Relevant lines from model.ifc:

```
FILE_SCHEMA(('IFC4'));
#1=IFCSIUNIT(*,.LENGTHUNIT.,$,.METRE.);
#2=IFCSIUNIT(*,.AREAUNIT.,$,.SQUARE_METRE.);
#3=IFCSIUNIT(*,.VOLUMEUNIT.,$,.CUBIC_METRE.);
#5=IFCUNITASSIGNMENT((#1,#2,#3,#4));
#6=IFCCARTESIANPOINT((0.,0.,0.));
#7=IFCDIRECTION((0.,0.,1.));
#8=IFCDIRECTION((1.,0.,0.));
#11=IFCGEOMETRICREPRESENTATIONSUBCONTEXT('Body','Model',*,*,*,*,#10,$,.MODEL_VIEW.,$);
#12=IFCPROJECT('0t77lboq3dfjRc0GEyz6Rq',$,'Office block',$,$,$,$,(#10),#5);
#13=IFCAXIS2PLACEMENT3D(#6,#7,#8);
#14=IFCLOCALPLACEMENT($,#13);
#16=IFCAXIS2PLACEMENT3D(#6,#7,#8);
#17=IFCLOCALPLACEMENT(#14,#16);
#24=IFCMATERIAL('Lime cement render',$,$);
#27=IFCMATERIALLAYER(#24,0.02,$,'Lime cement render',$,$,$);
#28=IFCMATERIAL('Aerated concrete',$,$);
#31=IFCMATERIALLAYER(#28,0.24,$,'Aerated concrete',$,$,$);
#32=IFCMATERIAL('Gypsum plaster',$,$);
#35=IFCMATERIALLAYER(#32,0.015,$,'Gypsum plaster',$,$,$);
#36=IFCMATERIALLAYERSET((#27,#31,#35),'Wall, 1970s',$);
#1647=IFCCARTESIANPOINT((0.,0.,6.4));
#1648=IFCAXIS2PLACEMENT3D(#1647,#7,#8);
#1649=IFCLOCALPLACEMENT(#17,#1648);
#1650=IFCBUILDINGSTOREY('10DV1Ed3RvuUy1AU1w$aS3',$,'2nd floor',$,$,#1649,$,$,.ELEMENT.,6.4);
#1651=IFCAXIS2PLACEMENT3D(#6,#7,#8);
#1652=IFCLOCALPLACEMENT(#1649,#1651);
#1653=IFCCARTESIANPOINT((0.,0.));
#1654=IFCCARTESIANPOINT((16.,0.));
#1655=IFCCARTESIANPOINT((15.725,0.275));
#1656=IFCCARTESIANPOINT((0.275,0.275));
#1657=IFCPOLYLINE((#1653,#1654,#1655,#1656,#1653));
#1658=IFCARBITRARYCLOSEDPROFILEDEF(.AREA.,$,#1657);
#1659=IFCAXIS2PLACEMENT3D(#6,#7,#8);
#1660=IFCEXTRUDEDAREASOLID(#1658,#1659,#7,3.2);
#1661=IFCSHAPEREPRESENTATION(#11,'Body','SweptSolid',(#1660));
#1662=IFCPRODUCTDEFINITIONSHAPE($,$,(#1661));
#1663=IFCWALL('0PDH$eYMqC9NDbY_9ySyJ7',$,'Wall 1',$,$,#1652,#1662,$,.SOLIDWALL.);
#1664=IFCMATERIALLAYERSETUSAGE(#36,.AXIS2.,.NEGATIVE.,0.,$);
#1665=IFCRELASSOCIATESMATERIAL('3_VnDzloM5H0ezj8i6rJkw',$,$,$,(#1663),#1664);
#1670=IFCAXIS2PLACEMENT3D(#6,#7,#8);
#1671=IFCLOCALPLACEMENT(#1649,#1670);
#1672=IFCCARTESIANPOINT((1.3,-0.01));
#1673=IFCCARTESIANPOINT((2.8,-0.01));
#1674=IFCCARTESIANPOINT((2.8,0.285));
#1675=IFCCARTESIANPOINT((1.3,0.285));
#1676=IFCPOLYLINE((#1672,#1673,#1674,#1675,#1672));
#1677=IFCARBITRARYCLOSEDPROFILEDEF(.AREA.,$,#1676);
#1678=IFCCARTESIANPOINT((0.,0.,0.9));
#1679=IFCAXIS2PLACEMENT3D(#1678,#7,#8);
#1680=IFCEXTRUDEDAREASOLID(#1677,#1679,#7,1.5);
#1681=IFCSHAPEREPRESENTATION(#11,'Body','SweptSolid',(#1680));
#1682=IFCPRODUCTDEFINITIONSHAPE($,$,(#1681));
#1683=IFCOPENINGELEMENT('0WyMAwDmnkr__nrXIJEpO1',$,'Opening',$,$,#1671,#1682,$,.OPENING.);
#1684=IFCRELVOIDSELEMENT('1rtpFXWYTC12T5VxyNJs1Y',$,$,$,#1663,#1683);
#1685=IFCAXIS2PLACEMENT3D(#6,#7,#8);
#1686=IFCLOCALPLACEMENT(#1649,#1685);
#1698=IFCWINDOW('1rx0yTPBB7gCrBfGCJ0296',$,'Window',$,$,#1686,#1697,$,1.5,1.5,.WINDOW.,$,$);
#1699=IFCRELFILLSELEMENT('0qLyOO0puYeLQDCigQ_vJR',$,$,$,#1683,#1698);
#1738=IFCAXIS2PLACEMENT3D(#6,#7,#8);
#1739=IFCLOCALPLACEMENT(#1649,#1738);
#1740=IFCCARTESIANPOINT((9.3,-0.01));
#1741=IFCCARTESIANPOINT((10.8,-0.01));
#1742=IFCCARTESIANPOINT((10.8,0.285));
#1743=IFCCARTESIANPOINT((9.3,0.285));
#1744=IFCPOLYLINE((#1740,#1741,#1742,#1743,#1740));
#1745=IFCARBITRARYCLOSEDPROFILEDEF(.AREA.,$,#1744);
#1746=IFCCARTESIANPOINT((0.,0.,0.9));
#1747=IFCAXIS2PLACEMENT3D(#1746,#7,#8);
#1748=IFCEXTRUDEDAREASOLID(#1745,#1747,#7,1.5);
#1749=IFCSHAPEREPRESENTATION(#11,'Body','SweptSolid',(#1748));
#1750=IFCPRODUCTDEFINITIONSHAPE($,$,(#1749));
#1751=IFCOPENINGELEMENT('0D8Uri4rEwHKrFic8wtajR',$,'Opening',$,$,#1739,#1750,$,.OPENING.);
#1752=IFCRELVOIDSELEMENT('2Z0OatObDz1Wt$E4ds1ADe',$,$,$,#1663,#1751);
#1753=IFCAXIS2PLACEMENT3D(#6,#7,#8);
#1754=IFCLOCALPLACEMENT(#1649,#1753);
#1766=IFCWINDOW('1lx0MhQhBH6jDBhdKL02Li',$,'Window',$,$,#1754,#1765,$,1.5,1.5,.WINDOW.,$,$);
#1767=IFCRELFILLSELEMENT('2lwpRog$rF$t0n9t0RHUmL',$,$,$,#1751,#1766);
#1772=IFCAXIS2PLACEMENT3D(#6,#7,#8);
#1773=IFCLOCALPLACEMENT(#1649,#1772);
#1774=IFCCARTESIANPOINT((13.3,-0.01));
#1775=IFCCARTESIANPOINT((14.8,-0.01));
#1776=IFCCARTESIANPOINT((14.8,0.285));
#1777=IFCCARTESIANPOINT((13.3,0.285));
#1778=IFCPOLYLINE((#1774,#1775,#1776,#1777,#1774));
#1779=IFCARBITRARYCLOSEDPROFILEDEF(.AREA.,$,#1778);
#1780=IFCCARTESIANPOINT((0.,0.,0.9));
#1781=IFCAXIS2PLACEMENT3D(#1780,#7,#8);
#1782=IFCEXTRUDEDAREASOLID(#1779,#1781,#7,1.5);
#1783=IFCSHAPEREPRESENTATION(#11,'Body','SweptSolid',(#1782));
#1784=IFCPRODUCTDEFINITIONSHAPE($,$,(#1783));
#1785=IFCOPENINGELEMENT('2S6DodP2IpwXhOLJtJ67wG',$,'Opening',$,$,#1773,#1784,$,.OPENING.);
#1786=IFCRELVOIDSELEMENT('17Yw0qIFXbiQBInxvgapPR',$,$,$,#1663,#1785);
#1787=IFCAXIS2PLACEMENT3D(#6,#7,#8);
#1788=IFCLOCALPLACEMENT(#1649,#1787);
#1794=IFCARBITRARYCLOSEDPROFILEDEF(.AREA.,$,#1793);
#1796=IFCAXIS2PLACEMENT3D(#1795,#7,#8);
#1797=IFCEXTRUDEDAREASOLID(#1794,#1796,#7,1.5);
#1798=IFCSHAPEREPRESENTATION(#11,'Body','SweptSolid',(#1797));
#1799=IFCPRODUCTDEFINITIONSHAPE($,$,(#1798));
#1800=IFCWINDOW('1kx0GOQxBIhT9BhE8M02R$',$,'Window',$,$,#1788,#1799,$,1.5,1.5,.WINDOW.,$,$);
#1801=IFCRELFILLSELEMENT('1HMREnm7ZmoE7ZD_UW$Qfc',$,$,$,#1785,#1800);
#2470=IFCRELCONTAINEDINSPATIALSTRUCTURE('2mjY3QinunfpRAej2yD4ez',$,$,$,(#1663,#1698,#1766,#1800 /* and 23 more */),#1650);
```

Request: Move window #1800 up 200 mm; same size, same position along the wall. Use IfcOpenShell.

```python
import numpy as np
import ifcopenshell
import ifcopenshell.api.geometry
import ifcopenshell.util.placement
import ifcopenshell.util.unit

model = ifcopenshell.open("model.ifc")
unit_scale = ifcopenshell.util.unit.calculate_unit_scale(model)

window = model.by_guid("1kx0GOQxBIhT9BhE8M02R$")
opening = window.FillsVoids[0].RelatingOpeningElement
dz = 0.2 / unit_scale

shift = np.array([0.0, 0.0, dz])
# The window is not placed relative to its opening, so move both.
for product in (opening, window):
    matrix = ifcopenshell.util.placement.get_local_placement(product.ObjectPlacement)
    matrix[:3, 3] += shift
    ifcopenshell.api.geometry.edit_object_placement(model, product=product, matrix=matrix, is_si=False)

print(f"moved by {dz * unit_scale:+.3f} m")

model.write("model_edited.ifc")
```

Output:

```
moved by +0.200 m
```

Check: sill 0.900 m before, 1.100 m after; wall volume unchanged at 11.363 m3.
